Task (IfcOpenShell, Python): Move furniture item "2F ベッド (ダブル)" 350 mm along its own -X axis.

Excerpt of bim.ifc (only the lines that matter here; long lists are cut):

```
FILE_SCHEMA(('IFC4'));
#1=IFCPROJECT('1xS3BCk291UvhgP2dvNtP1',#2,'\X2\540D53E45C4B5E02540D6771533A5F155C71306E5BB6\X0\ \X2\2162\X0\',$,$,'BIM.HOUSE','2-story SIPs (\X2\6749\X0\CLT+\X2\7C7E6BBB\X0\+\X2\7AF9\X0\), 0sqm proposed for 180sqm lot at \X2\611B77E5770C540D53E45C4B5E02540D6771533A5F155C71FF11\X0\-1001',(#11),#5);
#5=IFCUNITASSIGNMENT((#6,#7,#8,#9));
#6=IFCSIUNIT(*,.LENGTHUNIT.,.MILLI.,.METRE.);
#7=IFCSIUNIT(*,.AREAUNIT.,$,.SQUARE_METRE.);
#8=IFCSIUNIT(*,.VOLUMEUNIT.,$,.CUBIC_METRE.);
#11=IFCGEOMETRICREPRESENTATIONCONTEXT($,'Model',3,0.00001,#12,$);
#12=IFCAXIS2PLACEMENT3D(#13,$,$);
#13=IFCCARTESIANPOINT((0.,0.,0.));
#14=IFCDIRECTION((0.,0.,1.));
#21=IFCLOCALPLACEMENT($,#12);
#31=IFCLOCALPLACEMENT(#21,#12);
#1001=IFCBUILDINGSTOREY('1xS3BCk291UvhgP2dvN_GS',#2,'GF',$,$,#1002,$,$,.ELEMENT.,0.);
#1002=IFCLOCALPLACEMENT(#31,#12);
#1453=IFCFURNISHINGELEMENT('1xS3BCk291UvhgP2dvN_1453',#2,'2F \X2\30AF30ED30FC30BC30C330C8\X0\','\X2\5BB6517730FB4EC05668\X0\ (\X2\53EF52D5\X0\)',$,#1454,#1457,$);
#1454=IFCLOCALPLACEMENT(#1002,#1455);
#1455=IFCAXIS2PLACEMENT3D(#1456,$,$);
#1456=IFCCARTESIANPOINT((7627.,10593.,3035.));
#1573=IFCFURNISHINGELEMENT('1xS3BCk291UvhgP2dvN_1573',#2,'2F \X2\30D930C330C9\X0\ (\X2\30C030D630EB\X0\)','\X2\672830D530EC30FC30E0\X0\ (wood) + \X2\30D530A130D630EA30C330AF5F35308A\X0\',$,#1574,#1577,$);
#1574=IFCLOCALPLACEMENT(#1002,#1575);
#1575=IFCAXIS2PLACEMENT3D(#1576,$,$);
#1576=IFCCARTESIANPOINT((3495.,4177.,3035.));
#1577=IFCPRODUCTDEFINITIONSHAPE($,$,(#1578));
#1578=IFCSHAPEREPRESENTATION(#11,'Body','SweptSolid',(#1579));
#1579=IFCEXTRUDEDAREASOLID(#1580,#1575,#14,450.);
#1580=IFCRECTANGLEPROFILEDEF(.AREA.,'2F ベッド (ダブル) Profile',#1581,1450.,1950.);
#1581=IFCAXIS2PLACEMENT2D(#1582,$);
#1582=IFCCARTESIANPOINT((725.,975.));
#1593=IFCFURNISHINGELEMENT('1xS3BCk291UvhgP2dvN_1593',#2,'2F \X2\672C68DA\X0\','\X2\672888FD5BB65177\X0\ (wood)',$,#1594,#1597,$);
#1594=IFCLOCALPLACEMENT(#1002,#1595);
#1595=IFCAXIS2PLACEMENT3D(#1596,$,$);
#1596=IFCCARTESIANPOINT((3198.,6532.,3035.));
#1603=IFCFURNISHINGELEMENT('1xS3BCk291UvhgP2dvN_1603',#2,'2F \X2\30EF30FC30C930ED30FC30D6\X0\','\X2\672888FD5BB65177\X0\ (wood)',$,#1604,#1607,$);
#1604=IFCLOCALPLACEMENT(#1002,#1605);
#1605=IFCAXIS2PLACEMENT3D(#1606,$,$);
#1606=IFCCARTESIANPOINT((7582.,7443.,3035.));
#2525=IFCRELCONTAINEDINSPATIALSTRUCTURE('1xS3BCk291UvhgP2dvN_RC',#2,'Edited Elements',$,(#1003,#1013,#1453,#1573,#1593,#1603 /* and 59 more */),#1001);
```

```python
import ifcopenshell
import ifcopenshell.api.geometry
import ifcopenshell.util.placement
import ifcopenshell.util.unit

model = ifcopenshell.open("bim.ifc")
unit_scale = ifcopenshell.util.unit.calculate_unit_scale(model)

item = model.by_id(1573)
matrix = ifcopenshell.util.placement.get_local_placement(item.ObjectPlacement)
matrix[:3, 3] -= matrix[:3, 0] * 0.35 / unit_scale
ifcopenshell.api.geometry.edit_object_placement(model, product=item, matrix=matrix, is_si=False)

print(ifcopenshell.util.placement.get_local_placement(item.ObjectPlacement).round(3) + 0.0)

model.write("bim_edited.ifc")
```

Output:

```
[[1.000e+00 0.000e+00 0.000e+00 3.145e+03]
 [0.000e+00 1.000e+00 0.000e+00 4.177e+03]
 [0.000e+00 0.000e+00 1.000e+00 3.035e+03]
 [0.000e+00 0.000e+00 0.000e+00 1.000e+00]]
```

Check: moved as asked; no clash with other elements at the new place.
